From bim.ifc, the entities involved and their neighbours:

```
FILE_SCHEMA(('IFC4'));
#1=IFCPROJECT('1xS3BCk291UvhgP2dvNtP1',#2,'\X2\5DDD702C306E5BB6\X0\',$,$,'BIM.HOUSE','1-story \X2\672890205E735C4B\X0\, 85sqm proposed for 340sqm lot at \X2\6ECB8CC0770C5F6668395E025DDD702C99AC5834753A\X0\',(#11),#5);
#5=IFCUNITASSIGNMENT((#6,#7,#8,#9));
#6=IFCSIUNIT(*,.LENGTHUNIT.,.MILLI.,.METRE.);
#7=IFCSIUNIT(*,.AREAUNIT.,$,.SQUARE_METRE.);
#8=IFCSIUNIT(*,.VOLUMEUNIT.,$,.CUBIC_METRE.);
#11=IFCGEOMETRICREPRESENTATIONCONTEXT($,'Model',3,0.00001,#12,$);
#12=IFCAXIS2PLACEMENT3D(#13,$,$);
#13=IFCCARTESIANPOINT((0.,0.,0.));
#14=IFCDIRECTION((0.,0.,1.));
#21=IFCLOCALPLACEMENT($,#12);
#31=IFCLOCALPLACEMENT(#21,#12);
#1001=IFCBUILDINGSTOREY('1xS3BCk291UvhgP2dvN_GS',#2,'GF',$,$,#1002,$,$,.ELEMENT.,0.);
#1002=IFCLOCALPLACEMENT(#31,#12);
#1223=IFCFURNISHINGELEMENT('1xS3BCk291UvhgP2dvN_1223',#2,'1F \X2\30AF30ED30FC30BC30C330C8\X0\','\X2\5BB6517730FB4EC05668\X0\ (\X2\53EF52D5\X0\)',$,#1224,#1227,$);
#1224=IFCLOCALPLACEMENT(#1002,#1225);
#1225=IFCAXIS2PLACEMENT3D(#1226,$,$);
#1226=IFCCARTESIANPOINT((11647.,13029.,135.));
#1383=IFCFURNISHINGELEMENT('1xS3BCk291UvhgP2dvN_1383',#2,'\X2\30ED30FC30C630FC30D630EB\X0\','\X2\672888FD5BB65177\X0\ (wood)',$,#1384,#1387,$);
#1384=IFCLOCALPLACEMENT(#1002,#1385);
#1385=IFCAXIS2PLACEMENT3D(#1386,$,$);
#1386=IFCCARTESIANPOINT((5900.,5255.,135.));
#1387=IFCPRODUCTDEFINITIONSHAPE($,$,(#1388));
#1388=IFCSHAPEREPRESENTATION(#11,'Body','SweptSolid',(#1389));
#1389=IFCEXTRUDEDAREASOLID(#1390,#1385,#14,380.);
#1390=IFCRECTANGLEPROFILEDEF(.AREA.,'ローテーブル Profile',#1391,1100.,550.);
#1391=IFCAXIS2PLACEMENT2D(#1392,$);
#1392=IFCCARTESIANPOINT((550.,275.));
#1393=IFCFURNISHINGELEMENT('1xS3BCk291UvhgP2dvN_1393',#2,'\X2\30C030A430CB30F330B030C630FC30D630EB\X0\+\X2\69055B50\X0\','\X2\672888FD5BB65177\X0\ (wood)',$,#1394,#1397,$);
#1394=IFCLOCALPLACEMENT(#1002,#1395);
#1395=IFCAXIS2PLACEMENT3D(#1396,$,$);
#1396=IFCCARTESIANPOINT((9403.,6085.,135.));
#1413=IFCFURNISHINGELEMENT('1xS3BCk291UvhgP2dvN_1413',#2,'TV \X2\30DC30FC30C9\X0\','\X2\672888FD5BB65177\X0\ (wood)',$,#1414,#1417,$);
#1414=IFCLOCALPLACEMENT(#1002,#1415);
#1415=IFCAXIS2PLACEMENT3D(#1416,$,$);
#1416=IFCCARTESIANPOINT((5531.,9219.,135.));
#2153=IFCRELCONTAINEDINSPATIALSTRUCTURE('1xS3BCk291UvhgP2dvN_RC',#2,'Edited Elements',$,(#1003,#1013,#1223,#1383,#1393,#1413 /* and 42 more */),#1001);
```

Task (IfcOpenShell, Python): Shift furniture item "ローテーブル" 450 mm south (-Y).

```python
import ifcopenshell
import ifcopenshell.api.geometry
import ifcopenshell.util.placement
import ifcopenshell.util.unit

model = ifcopenshell.open("bim.ifc")
unit_scale = ifcopenshell.util.unit.calculate_unit_scale(model)

item = model.by_guid("1xS3BCk291UvhgP2dvN_1383")
matrix = ifcopenshell.util.placement.get_local_placement(item.ObjectPlacement)
matrix[1, 3] -= 0.45 / unit_scale
ifcopenshell.api.geometry.edit_object_placement(model, product=item, matrix=matrix, is_si=False)

print(ifcopenshell.util.placement.get_local_placement(item.ObjectPlacement).round(3) + 0.0)

model.write("bim_edited.ifc")
```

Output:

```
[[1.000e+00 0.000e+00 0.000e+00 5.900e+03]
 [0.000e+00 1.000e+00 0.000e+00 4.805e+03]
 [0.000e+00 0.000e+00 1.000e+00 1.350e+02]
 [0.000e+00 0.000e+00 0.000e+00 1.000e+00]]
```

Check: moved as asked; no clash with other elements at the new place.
